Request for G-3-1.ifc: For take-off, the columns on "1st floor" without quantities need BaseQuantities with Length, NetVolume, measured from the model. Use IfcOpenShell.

First a look at what the model holds.

```python
import ifcopenshell
import ifcopenshell.util.element
import ifcopenshell.util.unit

model = ifcopenshell.open("G-3-1.ifc")
print(model.schema)
for unit_type in ("LENGTHUNIT", "AREAUNIT", "VOLUMEUNIT"):
    print(unit_type, ifcopenshell.util.unit.calculate_unit_scale(model, unit_type))
storey = next(s for s in model.by_type("IfcBuildingStorey") if s.Name == "1st floor")
columns = [e for e in ifcopenshell.util.element.get_decomposition(storey) if e.is_a("IfcColumn")]
for e in sorted(columns, key=lambda e: e.id()):
    print(e.id(), e.is_a(), e.Name, list(ifcopenshell.util.element.get_psets(e, qtos_only=True)), sep=" | ")
```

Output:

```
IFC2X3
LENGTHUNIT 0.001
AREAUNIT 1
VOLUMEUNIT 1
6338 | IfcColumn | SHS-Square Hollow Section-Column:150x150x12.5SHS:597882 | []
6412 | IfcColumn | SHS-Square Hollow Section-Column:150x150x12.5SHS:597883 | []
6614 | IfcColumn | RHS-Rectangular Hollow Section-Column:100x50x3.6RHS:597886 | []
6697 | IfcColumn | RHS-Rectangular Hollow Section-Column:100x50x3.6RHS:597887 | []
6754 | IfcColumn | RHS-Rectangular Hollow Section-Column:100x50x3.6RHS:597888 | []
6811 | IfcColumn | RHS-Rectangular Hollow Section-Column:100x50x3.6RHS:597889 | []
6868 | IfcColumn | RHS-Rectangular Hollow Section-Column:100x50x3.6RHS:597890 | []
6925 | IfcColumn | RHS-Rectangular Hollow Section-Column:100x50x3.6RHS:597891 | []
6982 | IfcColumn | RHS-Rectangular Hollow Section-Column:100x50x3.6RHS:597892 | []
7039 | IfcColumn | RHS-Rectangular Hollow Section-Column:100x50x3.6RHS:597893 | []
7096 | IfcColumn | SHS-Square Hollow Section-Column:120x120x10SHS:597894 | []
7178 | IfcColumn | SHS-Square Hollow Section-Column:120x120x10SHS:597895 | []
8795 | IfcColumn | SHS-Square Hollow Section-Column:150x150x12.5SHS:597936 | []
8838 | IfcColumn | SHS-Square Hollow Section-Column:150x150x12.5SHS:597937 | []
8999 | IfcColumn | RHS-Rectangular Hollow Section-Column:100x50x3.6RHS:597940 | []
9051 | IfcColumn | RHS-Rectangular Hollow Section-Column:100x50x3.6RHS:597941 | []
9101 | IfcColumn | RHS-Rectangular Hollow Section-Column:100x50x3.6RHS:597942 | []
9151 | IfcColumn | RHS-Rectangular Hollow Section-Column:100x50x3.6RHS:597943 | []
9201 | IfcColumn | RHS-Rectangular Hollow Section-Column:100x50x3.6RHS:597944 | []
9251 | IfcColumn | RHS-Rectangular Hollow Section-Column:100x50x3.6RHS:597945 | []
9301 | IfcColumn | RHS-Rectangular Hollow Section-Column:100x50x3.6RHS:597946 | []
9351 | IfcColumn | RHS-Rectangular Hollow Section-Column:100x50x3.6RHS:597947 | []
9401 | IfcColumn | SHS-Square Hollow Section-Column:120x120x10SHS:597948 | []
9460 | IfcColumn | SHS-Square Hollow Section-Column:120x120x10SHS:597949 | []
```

```python
import ifcopenshell
import ifcopenshell.api.pset
import ifcopenshell.geom
import ifcopenshell.util.element
import ifcopenshell.util.shape
import ifcopenshell.util.unit

model = ifcopenshell.open("G-3-1.ifc")
unit_scale = ifcopenshell.util.unit.calculate_unit_scale(model)
volume_scale = ifcopenshell.util.unit.calculate_unit_scale(model, "VOLUMEUNIT")
settings = ifcopenshell.geom.settings()

storey = next(s for s in model.by_type("IfcBuildingStorey") if s.Name == "1st floor")
columns = [e for e in ifcopenshell.util.element.get_decomposition(storey) if e.is_a("IfcColumn")]

for e in sorted(columns, key=lambda e: e.id()):
    if ifcopenshell.util.element.get_psets(e, qtos_only=True, should_inherit=False):
        continue
    # Geometry comes back in metres, in the element's own axes.
    shape = ifcopenshell.geom.create_shape(settings, e)
    values = {
        "Length": ifcopenshell.util.shape.get_z(shape.geometry) / unit_scale,
        "NetVolume": ifcopenshell.util.shape.get_volume(shape.geometry) / volume_scale,
    }
    qto = ifcopenshell.api.pset.add_qto(model, product=e, name="BaseQuantities")
    ifcopenshell.api.pset.edit_qto(model, qto=qto, properties=values)
    print(e.id(), {k: round(v, 3) for k, v in values.items()})

model.write("G-3-1-out.ifc")
```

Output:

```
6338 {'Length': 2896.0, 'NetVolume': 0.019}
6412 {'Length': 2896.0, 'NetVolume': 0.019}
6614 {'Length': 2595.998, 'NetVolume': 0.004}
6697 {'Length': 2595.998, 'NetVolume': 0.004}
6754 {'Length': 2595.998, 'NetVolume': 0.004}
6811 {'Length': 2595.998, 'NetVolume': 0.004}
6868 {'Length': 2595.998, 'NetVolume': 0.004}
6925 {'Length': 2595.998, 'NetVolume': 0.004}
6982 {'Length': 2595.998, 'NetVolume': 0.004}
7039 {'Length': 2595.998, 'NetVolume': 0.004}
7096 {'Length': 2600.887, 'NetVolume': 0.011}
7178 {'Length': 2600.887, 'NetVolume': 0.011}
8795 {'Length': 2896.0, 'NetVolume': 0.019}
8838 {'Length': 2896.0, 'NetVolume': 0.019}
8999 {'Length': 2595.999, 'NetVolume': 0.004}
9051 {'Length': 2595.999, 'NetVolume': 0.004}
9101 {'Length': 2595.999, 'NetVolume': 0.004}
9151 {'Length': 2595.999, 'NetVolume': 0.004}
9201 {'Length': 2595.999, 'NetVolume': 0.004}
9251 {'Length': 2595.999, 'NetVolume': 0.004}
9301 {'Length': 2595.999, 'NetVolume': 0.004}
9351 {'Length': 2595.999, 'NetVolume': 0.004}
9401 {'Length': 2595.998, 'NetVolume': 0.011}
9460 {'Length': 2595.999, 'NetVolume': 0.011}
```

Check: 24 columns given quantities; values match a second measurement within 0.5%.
